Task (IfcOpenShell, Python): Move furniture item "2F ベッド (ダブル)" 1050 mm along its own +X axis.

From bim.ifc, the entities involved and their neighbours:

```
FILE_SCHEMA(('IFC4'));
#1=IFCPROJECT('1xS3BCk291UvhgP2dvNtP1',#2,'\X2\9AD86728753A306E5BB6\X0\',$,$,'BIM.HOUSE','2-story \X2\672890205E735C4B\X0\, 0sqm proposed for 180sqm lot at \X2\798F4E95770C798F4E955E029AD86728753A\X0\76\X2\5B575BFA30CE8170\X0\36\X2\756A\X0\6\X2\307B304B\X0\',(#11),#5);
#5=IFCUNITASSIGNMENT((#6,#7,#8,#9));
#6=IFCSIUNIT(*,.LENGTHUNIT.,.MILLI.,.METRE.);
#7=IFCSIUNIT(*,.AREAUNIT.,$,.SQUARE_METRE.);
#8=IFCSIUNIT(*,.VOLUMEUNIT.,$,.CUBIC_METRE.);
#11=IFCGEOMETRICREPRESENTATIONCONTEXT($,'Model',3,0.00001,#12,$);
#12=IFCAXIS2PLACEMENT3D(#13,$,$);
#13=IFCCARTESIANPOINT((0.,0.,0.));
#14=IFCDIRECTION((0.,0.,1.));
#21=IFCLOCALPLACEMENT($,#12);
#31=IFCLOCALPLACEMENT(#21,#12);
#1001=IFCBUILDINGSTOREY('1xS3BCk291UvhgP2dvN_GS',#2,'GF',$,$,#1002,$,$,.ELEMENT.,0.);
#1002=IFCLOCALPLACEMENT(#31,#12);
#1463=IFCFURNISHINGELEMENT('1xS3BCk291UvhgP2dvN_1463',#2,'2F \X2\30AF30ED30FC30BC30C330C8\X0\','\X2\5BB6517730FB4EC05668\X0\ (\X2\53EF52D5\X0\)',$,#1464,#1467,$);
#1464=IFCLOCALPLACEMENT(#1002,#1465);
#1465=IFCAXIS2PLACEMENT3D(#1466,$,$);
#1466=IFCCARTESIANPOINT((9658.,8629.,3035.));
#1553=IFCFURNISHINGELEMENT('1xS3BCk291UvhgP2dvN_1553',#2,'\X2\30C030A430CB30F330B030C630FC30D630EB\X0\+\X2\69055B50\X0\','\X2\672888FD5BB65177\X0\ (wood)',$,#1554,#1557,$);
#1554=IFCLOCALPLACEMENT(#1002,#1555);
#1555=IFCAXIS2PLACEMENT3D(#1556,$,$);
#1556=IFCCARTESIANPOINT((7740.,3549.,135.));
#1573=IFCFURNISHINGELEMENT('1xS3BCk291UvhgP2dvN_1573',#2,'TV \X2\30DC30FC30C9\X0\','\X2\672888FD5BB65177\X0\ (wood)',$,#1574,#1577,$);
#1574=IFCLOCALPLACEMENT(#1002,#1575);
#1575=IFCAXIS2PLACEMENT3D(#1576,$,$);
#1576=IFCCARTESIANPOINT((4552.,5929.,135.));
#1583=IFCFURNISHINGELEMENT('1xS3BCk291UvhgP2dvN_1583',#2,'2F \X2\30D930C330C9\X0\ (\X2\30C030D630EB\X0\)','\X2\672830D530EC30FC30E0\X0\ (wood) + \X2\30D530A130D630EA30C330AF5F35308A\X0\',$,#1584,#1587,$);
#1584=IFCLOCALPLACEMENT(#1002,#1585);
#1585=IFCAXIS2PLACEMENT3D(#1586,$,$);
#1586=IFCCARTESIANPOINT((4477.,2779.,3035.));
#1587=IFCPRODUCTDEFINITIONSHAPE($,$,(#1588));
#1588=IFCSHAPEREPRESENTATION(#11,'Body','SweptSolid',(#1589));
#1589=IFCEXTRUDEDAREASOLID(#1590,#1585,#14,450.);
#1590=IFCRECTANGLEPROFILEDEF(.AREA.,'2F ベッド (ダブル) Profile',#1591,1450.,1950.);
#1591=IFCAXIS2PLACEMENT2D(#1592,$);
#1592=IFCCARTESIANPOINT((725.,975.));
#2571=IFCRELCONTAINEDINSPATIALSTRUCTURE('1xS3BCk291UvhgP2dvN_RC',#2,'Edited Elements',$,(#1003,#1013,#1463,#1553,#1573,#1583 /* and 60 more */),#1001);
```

```python
import ifcopenshell
import ifcopenshell.api.geometry
import ifcopenshell.util.placement
import ifcopenshell.util.unit

model = ifcopenshell.open("bim.ifc")
unit_scale = ifcopenshell.util.unit.calculate_unit_scale(model)

item = model.by_guid("1xS3BCk291UvhgP2dvN_1583")
matrix = ifcopenshell.util.placement.get_local_placement(item.ObjectPlacement)
matrix[:3, 3] += matrix[:3, 0] * 1.05 / unit_scale
ifcopenshell.api.geometry.edit_object_placement(model, product=item, matrix=matrix, is_si=False)

print(ifcopenshell.util.placement.get_local_placement(item.ObjectPlacement).round(3) + 0.0)

model.write("bim_rev.ifc")
```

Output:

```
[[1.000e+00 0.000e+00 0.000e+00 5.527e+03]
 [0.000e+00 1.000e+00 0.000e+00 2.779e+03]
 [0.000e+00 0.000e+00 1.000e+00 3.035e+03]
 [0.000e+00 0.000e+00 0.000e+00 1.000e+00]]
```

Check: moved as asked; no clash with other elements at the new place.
